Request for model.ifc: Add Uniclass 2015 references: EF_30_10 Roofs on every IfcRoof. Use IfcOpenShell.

First a look at what the model holds.

```python
import ifcopenshell

model = ifcopenshell.open("model.ifc")
print(model.schema)
print("classifications:", [c.Name for c in model.by_type("IfcClassification")])
for ifc_class in ("IfcDoor", "IfcRoof", "IfcStair", "IfcWall", "IfcWindow"):
    print(ifc_class, len(model.by_type(ifc_class)))
```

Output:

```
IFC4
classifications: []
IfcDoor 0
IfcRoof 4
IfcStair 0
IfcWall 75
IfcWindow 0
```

```python
import ifcopenshell
import ifcopenshell.api.classification

model = ifcopenshell.open("model.ifc")

system = ifcopenshell.api.classification.add_classification(model, classification="Uniclass 2015")

codes = {
    "IfcRoof": ("EF_30_10", "Roofs"),
}
for ifc_class, (code, name) in codes.items():
    products = model.by_type(ifc_class)
    ifcopenshell.api.classification.add_reference(
        model, products=products, classification=system, identification=code, name=name
    )
    print(code, len(products))

model.write("model_rev.ifc")
```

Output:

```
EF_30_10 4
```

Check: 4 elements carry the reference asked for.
